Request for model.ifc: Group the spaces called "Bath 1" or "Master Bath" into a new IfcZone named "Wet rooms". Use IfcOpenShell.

First a look at what the model holds.

```python
import ifcopenshell

model = ifcopenshell.open("model.ifc")
print(model.schema)
seen = {}
for space in model.by_type("IfcSpace"):
    seen[space.LongName] = seen.get(space.LongName, 0) + 1
for name, count in sorted(seen.items(), key=str):
    print(count, "x", name)
print("zones:", [z.Name for z in model.by_type("IfcZone")][:20])
```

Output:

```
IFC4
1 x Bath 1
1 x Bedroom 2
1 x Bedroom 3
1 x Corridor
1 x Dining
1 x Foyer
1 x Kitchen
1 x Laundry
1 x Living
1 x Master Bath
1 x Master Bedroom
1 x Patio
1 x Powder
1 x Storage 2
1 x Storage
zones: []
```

```python
import ifcopenshell
import ifcopenshell.api.group
import ifcopenshell.api.root

model = ifcopenshell.open("model.ifc")

names = {"Bath 1", "Master Bath"}
spaces = [s for s in model.by_type("IfcSpace") if s.LongName in names]

zone = ifcopenshell.api.root.create_entity(model, ifc_class="IfcZone", name="Wet rooms")
ifcopenshell.api.group.assign_group(model, products=spaces, group=zone)
print(len(spaces), "spaces in", zone.Name)

model.write("model_updated.ifc")
```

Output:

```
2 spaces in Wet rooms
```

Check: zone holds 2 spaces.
